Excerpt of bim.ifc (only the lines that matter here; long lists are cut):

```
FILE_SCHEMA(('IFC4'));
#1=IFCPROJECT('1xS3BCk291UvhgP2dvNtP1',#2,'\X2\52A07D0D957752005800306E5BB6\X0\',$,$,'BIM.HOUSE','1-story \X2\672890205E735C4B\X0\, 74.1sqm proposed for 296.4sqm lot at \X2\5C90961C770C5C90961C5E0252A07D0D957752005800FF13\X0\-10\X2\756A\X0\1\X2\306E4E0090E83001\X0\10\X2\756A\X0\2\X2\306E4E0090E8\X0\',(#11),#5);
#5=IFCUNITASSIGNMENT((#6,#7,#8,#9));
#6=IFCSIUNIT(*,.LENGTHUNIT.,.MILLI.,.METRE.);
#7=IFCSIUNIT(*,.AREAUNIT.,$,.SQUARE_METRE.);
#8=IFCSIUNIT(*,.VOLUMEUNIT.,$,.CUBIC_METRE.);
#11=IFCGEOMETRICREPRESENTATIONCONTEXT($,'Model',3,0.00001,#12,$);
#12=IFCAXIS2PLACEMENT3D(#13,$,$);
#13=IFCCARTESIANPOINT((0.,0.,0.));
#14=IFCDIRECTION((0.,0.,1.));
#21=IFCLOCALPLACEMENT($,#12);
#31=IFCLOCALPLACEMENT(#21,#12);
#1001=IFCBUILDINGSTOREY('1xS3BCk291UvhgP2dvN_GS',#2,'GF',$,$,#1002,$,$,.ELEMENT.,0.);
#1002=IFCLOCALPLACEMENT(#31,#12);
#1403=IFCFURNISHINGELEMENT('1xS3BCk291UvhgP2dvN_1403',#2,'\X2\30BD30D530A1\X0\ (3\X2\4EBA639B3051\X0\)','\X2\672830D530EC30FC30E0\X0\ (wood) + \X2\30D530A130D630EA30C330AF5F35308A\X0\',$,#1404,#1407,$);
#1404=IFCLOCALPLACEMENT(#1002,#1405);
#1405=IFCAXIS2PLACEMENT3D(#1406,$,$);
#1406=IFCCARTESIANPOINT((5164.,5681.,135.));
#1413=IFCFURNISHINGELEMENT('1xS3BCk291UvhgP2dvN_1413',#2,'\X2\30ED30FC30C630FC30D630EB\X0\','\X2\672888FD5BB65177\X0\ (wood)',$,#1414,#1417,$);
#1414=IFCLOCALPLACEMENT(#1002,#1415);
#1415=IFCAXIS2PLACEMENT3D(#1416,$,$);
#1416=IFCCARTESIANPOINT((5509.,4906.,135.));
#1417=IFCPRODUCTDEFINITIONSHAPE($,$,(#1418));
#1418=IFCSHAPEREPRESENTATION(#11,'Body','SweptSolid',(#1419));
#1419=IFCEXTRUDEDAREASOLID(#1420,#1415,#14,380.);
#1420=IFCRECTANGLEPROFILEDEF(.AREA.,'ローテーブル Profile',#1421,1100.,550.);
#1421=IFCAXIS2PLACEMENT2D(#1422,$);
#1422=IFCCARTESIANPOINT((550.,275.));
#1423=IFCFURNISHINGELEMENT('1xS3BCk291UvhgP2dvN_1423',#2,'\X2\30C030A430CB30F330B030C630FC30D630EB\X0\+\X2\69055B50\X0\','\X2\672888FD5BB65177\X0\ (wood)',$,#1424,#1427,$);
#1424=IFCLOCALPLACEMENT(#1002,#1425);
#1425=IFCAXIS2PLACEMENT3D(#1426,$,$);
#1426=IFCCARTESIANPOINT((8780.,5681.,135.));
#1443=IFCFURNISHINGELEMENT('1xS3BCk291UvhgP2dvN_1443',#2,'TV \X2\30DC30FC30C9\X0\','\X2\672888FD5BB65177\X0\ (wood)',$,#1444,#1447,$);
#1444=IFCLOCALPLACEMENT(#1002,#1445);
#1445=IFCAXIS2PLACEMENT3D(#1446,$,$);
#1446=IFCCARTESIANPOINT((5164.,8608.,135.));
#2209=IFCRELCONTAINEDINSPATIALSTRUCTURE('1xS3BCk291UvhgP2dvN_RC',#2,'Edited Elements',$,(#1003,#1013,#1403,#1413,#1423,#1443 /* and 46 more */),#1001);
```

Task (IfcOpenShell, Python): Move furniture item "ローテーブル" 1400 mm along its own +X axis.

```python
import ifcopenshell
import ifcopenshell.api.geometry
import ifcopenshell.util.placement

model = ifcopenshell.open("bim.ifc")

item = model.by_guid("1xS3BCk291UvhgP2dvN_1413")
matrix = ifcopenshell.util.placement.get_local_placement(item.ObjectPlacement)
matrix[:3, 3] += matrix[:3, 0] * 1400.0
ifcopenshell.api.geometry.edit_object_placement(model, product=item, matrix=matrix, is_si=False)

print(ifcopenshell.util.placement.get_local_placement(item.ObjectPlacement).round(3) + 0.0)

model.write("bim_updated.ifc")
```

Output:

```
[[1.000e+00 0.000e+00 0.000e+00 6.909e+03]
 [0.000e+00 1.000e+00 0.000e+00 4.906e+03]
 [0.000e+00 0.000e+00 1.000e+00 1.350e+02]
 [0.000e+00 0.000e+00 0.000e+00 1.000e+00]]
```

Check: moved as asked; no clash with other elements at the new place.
